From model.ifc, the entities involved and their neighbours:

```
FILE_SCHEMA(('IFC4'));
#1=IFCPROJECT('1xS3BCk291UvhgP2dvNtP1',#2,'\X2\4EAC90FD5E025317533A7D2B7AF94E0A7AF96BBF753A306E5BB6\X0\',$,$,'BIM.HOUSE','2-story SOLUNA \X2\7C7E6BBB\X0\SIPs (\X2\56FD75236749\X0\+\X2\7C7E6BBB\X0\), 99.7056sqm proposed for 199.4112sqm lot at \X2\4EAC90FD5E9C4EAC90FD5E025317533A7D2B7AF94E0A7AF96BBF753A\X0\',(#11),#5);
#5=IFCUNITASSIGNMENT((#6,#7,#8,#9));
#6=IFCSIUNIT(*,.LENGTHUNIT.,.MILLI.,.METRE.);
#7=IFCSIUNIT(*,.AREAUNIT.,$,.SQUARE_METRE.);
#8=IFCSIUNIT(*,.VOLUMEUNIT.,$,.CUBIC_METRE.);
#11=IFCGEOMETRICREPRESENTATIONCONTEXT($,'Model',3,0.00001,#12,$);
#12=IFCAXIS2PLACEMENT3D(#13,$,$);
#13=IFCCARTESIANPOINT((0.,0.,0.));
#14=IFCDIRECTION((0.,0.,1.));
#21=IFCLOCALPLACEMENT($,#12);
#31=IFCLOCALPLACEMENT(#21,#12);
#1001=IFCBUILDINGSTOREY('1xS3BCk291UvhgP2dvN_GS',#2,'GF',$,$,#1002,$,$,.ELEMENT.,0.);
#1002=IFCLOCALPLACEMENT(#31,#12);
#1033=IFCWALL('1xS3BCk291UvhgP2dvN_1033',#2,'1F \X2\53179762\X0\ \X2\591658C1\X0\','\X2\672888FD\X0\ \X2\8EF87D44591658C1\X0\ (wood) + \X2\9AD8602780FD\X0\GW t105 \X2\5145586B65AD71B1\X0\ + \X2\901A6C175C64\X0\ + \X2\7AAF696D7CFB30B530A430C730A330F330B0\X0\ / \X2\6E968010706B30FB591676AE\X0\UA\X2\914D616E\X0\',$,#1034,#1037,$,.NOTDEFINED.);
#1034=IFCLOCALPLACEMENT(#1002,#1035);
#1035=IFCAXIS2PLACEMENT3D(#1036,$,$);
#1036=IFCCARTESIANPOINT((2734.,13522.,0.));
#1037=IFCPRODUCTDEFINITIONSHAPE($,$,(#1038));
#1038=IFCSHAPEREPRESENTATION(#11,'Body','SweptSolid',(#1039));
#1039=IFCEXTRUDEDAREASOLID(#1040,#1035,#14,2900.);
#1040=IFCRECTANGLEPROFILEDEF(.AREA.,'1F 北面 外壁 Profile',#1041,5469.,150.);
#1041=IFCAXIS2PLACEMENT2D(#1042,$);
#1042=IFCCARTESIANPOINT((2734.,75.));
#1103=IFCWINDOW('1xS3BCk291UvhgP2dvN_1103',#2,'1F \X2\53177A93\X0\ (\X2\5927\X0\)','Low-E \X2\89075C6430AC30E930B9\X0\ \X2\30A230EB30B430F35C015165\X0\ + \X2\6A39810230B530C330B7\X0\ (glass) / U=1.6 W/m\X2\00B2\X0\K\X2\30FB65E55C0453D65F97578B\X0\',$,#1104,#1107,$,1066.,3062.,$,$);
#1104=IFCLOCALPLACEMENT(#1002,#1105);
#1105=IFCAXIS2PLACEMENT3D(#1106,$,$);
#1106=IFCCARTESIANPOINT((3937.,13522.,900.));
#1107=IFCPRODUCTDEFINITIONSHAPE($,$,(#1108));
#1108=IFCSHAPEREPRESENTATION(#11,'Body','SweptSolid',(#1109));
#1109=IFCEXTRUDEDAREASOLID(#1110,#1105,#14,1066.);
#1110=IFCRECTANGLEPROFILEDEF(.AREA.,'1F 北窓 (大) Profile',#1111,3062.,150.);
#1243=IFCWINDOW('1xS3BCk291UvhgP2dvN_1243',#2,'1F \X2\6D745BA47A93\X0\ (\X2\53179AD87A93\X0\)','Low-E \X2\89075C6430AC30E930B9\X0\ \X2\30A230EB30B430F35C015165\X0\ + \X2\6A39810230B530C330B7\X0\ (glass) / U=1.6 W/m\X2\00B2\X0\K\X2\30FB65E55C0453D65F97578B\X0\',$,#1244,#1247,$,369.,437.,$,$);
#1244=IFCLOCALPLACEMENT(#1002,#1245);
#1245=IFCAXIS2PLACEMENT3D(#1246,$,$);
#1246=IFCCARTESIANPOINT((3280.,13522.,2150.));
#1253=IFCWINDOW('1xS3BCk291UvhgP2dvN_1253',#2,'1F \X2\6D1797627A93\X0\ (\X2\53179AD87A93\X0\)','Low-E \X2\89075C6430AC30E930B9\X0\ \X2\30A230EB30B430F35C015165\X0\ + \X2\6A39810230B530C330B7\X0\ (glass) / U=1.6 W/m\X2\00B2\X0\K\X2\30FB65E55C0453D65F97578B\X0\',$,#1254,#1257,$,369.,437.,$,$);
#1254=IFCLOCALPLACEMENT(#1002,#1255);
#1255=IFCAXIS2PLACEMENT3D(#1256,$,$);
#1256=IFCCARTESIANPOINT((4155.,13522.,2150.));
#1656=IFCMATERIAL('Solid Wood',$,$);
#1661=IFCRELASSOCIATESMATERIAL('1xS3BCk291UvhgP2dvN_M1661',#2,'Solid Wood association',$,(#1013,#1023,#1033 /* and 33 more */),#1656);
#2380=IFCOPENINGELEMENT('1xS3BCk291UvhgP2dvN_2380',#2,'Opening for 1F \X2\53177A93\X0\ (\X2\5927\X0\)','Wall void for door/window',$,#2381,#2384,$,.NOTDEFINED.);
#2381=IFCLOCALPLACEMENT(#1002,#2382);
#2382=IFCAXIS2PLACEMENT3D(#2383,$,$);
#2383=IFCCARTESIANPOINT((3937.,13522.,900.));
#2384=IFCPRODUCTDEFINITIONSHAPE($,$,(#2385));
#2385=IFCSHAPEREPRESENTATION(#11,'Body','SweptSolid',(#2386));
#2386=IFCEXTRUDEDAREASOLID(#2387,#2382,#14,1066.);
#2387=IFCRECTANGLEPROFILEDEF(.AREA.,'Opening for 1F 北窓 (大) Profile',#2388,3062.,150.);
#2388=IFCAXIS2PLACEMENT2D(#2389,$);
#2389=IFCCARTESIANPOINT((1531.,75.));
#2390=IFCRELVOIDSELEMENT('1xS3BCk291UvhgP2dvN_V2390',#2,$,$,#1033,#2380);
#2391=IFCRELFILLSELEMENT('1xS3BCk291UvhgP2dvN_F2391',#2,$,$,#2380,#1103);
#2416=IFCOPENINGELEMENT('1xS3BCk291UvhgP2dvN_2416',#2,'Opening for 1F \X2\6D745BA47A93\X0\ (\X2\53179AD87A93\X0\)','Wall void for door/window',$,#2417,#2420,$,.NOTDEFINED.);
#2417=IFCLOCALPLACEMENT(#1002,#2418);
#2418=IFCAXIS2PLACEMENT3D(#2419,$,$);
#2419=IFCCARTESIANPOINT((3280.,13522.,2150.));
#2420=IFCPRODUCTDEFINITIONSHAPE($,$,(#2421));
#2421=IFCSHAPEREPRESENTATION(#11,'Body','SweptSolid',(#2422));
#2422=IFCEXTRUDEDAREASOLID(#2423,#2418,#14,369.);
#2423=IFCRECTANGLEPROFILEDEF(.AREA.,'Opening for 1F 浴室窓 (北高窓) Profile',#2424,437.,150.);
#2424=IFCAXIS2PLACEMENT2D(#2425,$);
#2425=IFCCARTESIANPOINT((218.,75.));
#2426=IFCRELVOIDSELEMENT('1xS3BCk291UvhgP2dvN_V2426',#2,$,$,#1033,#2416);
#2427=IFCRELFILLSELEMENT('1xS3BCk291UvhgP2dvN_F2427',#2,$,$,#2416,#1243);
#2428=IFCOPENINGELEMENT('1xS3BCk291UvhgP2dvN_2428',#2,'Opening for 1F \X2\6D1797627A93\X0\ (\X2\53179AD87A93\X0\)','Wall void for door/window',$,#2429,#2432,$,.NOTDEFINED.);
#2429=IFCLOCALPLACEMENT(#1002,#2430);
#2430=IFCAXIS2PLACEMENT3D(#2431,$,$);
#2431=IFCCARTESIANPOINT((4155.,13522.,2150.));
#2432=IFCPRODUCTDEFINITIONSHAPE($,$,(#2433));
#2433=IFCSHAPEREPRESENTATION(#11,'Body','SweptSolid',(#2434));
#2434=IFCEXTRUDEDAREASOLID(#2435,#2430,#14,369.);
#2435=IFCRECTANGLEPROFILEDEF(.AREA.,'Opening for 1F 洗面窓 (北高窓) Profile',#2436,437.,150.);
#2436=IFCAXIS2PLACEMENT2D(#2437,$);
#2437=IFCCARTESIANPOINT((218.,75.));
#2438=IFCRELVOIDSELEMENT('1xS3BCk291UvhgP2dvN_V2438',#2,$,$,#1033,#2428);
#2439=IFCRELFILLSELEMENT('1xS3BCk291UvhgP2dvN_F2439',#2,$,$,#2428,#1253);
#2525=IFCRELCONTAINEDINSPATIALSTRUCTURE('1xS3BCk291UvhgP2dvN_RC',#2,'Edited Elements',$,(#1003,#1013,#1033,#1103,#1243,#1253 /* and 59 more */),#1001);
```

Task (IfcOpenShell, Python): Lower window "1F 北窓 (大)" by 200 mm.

```python
import numpy as np
import ifcopenshell
import ifcopenshell.api.geometry
import ifcopenshell.util.placement
import ifcopenshell.util.unit

model = ifcopenshell.open("model.ifc")
unit_scale = ifcopenshell.util.unit.calculate_unit_scale(model)

window = model.by_guid("1xS3BCk291UvhgP2dvN_1103")
opening = window.FillsVoids[0].RelatingOpeningElement
dz = -0.2 / unit_scale

shift = np.array([0.0, 0.0, dz])
# The window is not placed relative to its opening, so move both.
for product in (opening, window):
    matrix = ifcopenshell.util.placement.get_local_placement(product.ObjectPlacement)
    matrix[:3, 3] += shift
    ifcopenshell.api.geometry.edit_object_placement(model, product=product, matrix=matrix, is_si=False)

print(f"moved by {dz * unit_scale:+.3f} m")

model.write("model_edited.ifc")
```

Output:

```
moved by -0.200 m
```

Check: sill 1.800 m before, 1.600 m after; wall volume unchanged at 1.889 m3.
